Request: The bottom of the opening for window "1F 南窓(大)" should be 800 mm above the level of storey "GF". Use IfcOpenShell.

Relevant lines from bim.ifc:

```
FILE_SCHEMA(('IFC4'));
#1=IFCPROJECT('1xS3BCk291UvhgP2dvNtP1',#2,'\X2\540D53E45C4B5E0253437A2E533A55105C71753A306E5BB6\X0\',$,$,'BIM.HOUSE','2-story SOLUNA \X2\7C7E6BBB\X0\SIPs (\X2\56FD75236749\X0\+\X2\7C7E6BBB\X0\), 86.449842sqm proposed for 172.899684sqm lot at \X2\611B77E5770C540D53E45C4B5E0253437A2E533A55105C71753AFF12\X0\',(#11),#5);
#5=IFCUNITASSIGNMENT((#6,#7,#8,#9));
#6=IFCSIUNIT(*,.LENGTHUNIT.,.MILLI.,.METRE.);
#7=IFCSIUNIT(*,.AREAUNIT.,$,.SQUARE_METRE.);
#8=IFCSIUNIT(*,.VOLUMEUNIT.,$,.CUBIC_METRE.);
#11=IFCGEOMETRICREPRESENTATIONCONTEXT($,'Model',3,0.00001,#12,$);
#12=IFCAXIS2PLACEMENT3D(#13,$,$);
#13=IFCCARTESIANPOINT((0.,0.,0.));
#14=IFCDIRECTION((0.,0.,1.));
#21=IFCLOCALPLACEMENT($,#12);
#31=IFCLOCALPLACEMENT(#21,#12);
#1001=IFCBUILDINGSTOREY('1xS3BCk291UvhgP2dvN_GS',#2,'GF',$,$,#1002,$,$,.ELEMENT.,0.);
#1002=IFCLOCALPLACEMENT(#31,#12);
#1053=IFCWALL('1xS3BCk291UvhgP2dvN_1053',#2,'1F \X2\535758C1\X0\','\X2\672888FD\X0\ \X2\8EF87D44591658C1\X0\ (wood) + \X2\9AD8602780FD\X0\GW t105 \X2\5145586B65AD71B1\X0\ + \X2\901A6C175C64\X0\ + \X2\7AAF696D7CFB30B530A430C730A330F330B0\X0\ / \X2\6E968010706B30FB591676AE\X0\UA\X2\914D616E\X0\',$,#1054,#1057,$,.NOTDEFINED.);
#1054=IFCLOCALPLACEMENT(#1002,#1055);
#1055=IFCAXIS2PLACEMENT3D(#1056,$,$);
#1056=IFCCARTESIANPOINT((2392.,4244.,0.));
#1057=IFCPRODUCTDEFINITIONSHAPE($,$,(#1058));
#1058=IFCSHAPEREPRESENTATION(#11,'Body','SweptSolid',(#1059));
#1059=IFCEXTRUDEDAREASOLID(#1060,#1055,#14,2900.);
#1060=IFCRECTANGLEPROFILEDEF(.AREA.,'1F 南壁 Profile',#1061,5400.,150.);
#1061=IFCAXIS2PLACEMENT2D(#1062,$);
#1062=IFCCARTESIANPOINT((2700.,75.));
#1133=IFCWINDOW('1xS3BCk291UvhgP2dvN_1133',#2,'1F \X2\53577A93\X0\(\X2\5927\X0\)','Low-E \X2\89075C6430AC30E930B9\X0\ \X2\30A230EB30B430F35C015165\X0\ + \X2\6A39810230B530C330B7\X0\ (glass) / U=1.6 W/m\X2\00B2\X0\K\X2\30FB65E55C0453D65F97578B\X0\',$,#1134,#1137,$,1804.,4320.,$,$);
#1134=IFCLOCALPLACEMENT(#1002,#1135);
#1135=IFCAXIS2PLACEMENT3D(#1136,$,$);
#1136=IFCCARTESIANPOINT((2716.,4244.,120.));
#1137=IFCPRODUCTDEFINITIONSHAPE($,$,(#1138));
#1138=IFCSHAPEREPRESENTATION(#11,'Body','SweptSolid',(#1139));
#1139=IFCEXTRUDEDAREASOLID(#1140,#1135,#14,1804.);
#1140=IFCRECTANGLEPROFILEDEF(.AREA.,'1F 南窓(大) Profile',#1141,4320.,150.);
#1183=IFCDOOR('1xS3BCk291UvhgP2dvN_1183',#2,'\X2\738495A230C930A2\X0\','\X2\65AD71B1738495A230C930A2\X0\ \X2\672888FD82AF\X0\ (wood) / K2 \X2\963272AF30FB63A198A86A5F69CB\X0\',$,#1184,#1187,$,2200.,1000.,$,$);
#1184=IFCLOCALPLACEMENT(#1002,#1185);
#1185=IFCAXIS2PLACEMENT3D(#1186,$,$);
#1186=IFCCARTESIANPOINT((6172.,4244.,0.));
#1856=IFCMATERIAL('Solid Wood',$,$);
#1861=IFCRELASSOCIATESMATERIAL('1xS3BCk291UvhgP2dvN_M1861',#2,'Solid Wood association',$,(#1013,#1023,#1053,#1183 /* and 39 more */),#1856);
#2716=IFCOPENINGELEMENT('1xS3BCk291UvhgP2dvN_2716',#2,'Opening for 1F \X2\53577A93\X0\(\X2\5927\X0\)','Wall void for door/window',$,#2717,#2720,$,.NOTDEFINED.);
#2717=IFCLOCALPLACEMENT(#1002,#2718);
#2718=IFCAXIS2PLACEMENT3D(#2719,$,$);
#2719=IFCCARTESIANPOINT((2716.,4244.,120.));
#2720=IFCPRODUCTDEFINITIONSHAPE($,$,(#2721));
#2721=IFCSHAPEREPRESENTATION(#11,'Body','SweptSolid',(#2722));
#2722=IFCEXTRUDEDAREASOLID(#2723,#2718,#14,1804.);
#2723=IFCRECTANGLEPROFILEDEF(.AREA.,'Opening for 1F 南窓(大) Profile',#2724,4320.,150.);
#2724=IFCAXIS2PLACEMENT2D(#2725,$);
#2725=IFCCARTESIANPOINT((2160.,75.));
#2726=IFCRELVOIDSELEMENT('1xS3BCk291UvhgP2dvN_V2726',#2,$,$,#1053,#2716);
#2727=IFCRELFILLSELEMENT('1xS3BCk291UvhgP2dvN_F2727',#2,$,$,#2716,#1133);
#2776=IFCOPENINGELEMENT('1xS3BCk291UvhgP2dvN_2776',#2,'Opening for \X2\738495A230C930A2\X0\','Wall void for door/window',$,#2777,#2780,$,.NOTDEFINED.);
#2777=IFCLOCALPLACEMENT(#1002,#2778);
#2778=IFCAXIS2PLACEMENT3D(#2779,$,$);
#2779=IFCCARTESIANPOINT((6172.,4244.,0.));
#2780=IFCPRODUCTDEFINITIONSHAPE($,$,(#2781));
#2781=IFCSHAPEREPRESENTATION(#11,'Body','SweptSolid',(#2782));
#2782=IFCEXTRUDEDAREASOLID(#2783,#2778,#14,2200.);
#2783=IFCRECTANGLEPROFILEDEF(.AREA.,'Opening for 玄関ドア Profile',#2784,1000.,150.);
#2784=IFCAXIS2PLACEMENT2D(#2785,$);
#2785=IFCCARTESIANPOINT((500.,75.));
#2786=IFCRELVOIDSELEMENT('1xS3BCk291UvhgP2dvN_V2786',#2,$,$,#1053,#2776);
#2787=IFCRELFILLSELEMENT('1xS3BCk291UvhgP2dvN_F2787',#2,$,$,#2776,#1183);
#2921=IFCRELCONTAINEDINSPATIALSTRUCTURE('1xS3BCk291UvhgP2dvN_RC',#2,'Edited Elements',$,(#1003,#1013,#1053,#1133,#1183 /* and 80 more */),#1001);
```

```python
import numpy as np
import ifcopenshell
import ifcopenshell.api.geometry
import ifcopenshell.geom
import ifcopenshell.util.element
import ifcopenshell.util.placement
import ifcopenshell.util.shape
import ifcopenshell.util.unit

model = ifcopenshell.open("bim.ifc")
unit_scale = ifcopenshell.util.unit.calculate_unit_scale(model)

window = model.by_guid("1xS3BCk291UvhgP2dvN_1133")
opening = window.FillsVoids[0].RelatingOpeningElement
storey = ifcopenshell.util.element.get_container(window, ifc_class="IfcBuildingStorey")
level = ifcopenshell.util.placement.get_local_placement(storey.ObjectPlacement)[2, 3]

# The opening's origin need not be at the sill, so measure its lowest point.
shape = ifcopenshell.geom.create_shape(ifcopenshell.geom.settings(), opening)
bottom = ifcopenshell.util.shape.get_shape_bottom_elevation(shape, shape.geometry) / unit_scale
dz = level + 0.8 / unit_scale - bottom

shift = np.array([0.0, 0.0, dz])
# The window is not placed relative to its opening, so move both.
for product in (opening, window):
    matrix = ifcopenshell.util.placement.get_local_placement(product.ObjectPlacement)
    matrix[:3, 3] += shift
    ifcopenshell.api.geometry.edit_object_placement(model, product=product, matrix=matrix, is_si=False)

print(f"moved by {dz * unit_scale:+.3f} m")

model.write("bim-out.ifc")
```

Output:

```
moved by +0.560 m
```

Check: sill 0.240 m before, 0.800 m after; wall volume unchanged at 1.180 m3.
